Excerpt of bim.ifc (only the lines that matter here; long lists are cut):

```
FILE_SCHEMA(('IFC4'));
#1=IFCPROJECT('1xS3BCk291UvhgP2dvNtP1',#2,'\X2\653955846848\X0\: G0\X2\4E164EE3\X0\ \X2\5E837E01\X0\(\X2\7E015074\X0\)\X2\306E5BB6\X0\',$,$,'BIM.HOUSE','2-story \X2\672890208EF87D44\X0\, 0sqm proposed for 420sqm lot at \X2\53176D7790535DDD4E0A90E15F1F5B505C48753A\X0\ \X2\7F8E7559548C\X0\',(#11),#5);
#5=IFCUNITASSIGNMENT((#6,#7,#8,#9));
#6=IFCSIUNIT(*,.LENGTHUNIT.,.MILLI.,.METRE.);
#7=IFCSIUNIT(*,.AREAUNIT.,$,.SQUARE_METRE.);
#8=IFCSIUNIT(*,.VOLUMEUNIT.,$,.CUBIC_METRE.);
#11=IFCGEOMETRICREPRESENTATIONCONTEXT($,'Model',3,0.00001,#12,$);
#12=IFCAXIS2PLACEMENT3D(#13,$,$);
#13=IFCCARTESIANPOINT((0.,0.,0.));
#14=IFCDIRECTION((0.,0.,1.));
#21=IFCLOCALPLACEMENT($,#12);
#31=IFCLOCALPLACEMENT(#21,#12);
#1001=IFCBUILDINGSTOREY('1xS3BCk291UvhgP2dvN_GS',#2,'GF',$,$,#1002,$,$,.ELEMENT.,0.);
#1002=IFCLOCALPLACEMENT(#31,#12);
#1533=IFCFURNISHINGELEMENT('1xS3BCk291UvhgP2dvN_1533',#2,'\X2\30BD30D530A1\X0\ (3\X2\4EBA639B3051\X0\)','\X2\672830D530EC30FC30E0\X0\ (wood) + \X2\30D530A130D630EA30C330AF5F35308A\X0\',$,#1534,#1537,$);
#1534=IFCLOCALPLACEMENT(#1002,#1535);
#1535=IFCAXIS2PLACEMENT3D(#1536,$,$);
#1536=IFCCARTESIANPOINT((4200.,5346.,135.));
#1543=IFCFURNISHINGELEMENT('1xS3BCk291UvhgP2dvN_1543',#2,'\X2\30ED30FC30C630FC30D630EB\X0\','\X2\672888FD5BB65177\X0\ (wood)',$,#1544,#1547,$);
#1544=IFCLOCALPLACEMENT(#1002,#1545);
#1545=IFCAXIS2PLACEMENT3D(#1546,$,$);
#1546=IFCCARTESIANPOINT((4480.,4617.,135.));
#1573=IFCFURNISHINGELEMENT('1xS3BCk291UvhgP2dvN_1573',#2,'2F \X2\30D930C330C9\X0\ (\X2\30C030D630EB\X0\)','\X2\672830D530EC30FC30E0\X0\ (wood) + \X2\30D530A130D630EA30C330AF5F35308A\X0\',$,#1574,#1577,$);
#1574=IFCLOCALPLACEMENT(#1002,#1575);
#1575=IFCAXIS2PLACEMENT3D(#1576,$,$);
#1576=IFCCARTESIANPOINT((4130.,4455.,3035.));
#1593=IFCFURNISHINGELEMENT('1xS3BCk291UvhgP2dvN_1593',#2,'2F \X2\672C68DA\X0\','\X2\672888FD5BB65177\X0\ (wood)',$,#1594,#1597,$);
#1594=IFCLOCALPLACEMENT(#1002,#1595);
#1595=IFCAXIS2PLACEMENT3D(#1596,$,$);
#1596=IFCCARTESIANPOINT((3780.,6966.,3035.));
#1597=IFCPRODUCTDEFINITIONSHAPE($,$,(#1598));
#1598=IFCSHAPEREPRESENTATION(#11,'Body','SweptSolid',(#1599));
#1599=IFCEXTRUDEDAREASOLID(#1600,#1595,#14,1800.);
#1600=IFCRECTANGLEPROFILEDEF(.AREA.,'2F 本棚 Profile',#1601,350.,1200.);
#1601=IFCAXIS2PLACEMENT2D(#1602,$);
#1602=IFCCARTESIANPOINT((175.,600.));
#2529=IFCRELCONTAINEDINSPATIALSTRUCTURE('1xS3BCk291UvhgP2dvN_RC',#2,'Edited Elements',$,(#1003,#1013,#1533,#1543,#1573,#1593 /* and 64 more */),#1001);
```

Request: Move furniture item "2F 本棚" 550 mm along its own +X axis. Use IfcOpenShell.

```python
import ifcopenshell
import ifcopenshell.api.geometry
import ifcopenshell.util.placement
import ifcopenshell.util.unit

model = ifcopenshell.open("bim.ifc")
unit_scale = ifcopenshell.util.unit.calculate_unit_scale(model)

item = model.by_id(1593)
matrix = ifcopenshell.util.placement.get_local_placement(item.ObjectPlacement)
matrix[:3, 3] += matrix[:3, 0] * 0.55 / unit_scale
ifcopenshell.api.geometry.edit_object_placement(model, product=item, matrix=matrix, is_si=False)

print(ifcopenshell.util.placement.get_local_placement(item.ObjectPlacement).round(3) + 0.0)

model.write("bim-out.ifc")
```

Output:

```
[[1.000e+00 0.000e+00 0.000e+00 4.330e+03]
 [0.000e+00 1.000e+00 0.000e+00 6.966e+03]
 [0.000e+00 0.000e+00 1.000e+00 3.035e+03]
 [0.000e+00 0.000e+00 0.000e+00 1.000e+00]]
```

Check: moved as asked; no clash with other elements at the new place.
